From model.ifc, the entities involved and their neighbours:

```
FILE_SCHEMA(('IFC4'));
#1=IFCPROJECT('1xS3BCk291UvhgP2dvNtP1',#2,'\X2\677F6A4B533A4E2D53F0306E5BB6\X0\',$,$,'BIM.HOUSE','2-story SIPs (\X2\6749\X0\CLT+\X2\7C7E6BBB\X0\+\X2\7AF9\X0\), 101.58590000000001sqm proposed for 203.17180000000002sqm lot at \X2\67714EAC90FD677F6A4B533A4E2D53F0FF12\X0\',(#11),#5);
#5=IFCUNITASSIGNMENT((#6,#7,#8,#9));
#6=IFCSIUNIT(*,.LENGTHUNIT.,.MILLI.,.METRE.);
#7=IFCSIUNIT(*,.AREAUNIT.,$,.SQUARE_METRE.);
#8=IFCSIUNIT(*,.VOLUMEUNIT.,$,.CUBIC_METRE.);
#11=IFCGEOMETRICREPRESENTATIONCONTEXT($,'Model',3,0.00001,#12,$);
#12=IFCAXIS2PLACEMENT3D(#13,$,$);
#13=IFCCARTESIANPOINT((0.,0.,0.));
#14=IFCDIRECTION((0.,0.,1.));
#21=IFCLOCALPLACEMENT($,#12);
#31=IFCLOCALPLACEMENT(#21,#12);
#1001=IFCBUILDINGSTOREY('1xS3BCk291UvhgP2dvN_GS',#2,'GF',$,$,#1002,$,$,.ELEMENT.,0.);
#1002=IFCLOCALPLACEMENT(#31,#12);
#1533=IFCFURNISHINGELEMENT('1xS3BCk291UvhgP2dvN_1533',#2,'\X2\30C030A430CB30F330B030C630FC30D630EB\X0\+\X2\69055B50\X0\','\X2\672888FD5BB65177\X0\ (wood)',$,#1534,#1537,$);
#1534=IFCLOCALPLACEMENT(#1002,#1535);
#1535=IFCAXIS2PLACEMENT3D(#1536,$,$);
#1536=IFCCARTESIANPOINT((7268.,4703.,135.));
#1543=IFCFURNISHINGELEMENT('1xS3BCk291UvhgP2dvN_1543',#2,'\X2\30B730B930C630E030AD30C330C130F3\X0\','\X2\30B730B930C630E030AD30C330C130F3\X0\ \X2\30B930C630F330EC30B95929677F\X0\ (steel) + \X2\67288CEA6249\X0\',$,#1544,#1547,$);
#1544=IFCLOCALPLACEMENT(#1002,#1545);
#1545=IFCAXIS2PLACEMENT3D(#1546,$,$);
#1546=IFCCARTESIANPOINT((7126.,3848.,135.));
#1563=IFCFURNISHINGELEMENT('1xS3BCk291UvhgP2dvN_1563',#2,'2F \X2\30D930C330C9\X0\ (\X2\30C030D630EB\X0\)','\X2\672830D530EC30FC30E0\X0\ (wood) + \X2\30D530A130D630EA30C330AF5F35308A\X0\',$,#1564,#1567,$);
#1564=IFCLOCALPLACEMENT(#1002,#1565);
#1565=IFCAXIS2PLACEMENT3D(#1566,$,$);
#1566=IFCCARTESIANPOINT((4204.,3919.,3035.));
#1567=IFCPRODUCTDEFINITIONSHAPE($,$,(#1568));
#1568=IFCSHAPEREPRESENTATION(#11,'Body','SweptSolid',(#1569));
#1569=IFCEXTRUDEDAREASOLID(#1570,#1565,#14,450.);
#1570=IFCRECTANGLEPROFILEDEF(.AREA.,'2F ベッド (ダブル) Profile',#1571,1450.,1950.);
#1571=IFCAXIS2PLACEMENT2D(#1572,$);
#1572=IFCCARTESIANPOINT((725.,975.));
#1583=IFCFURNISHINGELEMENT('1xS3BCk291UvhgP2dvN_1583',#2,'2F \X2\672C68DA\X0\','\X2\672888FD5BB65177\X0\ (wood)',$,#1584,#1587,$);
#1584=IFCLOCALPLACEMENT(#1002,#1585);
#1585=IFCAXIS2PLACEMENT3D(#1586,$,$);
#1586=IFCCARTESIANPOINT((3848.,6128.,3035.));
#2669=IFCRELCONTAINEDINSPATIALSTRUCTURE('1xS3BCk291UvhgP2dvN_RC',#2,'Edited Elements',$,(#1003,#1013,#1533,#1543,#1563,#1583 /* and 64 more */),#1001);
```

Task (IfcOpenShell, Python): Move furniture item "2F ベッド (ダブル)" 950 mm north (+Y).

```python
import ifcopenshell
import ifcopenshell.api.geometry
import ifcopenshell.util.placement
import ifcopenshell.util.unit

model = ifcopenshell.open("model.ifc")
unit_scale = ifcopenshell.util.unit.calculate_unit_scale(model)

item = model.by_guid("1xS3BCk291UvhgP2dvN_1563")
matrix = ifcopenshell.util.placement.get_local_placement(item.ObjectPlacement)
matrix[1, 3] += 0.95 / unit_scale
ifcopenshell.api.geometry.edit_object_placement(model, product=item, matrix=matrix, is_si=False)

print(ifcopenshell.util.placement.get_local_placement(item.ObjectPlacement).round(3) + 0.0)

model.write("model_rev.ifc")
```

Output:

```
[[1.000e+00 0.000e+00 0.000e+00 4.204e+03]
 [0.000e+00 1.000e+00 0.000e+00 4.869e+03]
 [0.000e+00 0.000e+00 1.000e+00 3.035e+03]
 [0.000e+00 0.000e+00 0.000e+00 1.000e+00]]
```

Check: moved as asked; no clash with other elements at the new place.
